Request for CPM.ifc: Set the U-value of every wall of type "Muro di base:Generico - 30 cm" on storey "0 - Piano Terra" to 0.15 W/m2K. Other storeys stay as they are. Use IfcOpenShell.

First a look at what the model holds.

```python
import ifcopenshell
import ifcopenshell.util.element

model = ifcopenshell.open("CPM.ifc")
print(model.schema)
storey = next(s for s in model.by_type("IfcBuildingStorey") if s.Name == "0 - Piano Terra")
walls = [e for e in ifcopenshell.util.element.get_decomposition(storey) if e.is_a("IfcWall")]
seen = {}
for e in walls:
    element_type = ifcopenshell.util.element.get_type(e)
    key = (element_type.Name if element_type != e and element_type else None, ifcopenshell.util.element.get_pset(e, "Pset_WallCommon", "ThermalTransmittance"))
    seen[key] = seen.get(key, 0) + 1
for (name, value), count in sorted(seen.items(), key=str):
    print(count, "x", name, "|", value)
```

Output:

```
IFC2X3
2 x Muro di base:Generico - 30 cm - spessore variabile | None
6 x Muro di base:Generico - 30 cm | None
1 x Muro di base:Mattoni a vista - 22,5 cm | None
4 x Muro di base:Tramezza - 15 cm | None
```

```python
import ifcopenshell
import ifcopenshell.api.pset
import ifcopenshell.util.element

model = ifcopenshell.open("CPM.ifc")

storey = next(s for s in model.by_type("IfcBuildingStorey") if s.Name == "0 - Piano Terra")
walls = [e for e in ifcopenshell.util.element.get_decomposition(storey) if e.is_a("IfcWall")]

count = 0
for e in walls:
    element_type = ifcopenshell.util.element.get_type(e)
    if element_type in (None, e) or element_type.Name != "Muro di base:Generico - 30 cm":
        continue
    # add_pset returns the element's existing set when there is one.
    pset = ifcopenshell.api.pset.add_pset(model, product=e, name="Pset_WallCommon")
    ifcopenshell.api.pset.edit_pset(model, pset=pset, properties={"ThermalTransmittance": 0.15})
    count += 1

print(count, "walls updated")

model.write("CPM_updated.ifc")
```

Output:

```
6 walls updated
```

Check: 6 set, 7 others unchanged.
